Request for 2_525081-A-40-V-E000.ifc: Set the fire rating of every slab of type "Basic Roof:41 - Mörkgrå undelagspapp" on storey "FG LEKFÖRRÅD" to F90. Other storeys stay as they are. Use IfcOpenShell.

First a look at what the model holds.

```python
import ifcopenshell
import ifcopenshell.util.element

model = ifcopenshell.open("2_525081-A-40-V-E000.ifc")
print(model.schema)
storey = next(s for s in model.by_type("IfcBuildingStorey") if s.Name == "FG LEKFÖRRÅD")
slabs = [e for e in ifcopenshell.util.element.get_decomposition(storey) if e.is_a("IfcSlab")]
seen = {}
for e in slabs:
    element_type = ifcopenshell.util.element.get_type(e)
    key = (element_type.Name if element_type != e and element_type else None, ifcopenshell.util.element.get_pset(e, "Pset_SlabCommon", "FireRating"))
    seen[key] = seen.get(key, 0) + 1
for (name, value), count in sorted(seen.items(), key=str):
    print(count, "x", name, "|", value)
```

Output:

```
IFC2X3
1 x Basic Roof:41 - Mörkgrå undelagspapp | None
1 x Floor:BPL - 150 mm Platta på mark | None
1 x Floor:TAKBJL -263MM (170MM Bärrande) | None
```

```python
import ifcopenshell
import ifcopenshell.api.pset
import ifcopenshell.util.element

model = ifcopenshell.open("2_525081-A-40-V-E000.ifc")

storey = next(s for s in model.by_type("IfcBuildingStorey") if s.Name == "FG LEKFÖRRÅD")
slabs = [e for e in ifcopenshell.util.element.get_decomposition(storey) if e.is_a("IfcSlab")]

count = 0
for e in slabs:
    element_type = ifcopenshell.util.element.get_type(e)
    if element_type in (None, e) or element_type.Name != "Basic Roof:41 - Mörkgrå undelagspapp":
        continue
    # add_pset returns the element's existing set when there is one.
    pset = ifcopenshell.api.pset.add_pset(model, product=e, name="Pset_SlabCommon")
    ifcopenshell.api.pset.edit_pset(model, pset=pset, properties={"FireRating": "F90"})
    count += 1

print(count, "slabs updated")

model.write("2_525081-A-40-V-E000_rev.ifc")
```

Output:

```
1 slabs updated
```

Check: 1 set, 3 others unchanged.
